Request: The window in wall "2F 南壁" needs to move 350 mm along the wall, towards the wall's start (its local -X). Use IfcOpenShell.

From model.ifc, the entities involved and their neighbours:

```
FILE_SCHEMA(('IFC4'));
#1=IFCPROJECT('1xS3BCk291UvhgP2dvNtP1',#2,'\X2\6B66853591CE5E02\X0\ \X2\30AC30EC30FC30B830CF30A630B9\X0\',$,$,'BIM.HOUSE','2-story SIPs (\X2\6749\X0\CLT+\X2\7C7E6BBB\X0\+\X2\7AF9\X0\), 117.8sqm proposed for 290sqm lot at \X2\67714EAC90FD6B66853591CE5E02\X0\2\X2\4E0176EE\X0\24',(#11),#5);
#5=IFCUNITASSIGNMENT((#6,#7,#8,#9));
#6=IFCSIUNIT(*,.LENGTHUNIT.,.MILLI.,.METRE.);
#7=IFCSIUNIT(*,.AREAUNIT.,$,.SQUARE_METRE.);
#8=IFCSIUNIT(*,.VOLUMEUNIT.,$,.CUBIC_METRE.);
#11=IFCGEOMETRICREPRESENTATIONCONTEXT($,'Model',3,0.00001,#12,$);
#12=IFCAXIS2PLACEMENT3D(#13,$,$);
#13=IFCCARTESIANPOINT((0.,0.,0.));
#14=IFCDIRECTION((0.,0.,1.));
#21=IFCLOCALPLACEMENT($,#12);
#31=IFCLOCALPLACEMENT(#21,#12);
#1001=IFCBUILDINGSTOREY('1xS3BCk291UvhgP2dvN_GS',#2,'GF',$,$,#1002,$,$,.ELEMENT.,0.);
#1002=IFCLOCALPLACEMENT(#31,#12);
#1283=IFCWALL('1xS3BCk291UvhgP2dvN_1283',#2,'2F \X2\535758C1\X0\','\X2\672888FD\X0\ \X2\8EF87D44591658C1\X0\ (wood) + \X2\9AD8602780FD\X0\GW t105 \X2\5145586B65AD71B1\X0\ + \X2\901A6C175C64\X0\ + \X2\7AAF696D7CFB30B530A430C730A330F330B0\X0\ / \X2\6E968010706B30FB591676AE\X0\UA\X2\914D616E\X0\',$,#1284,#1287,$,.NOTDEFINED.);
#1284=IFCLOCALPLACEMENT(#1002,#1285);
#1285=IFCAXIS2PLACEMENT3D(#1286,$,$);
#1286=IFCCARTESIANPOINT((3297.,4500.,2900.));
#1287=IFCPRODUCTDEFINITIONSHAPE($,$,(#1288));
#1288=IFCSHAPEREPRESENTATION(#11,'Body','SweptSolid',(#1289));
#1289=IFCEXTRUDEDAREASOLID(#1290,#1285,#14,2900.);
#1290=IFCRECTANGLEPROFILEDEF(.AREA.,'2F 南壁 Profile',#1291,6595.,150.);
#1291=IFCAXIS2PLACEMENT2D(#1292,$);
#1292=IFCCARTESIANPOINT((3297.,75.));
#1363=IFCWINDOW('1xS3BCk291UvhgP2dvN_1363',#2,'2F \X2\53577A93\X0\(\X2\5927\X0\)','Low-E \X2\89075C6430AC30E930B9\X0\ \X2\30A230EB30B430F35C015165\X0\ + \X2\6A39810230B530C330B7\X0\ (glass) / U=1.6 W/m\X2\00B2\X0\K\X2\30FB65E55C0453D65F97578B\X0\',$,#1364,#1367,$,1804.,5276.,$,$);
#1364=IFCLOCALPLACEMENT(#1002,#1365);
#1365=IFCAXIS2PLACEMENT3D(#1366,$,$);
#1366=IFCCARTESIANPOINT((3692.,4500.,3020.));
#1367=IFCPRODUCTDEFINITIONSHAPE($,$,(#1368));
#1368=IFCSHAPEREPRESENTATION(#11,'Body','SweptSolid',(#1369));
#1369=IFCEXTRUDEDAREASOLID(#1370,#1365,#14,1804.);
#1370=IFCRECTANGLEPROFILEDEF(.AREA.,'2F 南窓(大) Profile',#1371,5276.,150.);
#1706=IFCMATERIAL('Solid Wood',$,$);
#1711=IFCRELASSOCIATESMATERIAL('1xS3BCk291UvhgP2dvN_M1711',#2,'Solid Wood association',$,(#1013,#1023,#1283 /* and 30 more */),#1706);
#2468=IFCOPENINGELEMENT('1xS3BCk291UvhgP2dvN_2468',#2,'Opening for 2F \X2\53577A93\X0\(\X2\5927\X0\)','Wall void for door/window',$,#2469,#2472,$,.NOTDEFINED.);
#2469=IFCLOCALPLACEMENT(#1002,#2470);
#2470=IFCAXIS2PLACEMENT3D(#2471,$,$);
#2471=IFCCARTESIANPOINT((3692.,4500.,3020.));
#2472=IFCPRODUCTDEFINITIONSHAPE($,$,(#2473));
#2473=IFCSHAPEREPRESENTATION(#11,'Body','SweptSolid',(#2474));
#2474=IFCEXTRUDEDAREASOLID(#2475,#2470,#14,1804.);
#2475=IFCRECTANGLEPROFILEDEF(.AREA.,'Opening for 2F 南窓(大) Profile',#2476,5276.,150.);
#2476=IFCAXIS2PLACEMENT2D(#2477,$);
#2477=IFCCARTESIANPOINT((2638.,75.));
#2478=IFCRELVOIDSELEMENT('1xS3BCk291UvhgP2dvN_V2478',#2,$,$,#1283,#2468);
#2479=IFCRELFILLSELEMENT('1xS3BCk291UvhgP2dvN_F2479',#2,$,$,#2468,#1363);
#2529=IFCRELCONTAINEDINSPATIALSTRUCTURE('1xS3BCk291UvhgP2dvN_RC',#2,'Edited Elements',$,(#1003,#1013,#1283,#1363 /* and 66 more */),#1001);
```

```python
import ifcopenshell
import ifcopenshell.api.geometry
import ifcopenshell.util.placement
import ifcopenshell.util.unit

model = ifcopenshell.open("model.ifc")
unit_scale = ifcopenshell.util.unit.calculate_unit_scale(model)

window = model.by_id(1363)
opening = window.FillsVoids[0].RelatingOpeningElement
wall = opening.VoidsElements[0].RelatingBuildingElement

wall_matrix = ifcopenshell.util.placement.get_local_placement(wall.ObjectPlacement)
shift = wall_matrix[:3, 0] * -0.35 / unit_scale
before = ifcopenshell.util.placement.get_local_placement(window.ObjectPlacement)[:3, 3].copy()

# The window is not placed relative to its opening, so move both.
for product in (opening, window):
    matrix = ifcopenshell.util.placement.get_local_placement(product.ObjectPlacement)
    matrix[:3, 3] += shift
    ifcopenshell.api.geometry.edit_object_placement(model, product=product, matrix=matrix, is_si=False)

after = ifcopenshell.util.placement.get_local_placement(window.ObjectPlacement)[:3, 3]
print("window moved by", (after - before).round(3) + 0.0)

model.write("model_rev.ifc")
```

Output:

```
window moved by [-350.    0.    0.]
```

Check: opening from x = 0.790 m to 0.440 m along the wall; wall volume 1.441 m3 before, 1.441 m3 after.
